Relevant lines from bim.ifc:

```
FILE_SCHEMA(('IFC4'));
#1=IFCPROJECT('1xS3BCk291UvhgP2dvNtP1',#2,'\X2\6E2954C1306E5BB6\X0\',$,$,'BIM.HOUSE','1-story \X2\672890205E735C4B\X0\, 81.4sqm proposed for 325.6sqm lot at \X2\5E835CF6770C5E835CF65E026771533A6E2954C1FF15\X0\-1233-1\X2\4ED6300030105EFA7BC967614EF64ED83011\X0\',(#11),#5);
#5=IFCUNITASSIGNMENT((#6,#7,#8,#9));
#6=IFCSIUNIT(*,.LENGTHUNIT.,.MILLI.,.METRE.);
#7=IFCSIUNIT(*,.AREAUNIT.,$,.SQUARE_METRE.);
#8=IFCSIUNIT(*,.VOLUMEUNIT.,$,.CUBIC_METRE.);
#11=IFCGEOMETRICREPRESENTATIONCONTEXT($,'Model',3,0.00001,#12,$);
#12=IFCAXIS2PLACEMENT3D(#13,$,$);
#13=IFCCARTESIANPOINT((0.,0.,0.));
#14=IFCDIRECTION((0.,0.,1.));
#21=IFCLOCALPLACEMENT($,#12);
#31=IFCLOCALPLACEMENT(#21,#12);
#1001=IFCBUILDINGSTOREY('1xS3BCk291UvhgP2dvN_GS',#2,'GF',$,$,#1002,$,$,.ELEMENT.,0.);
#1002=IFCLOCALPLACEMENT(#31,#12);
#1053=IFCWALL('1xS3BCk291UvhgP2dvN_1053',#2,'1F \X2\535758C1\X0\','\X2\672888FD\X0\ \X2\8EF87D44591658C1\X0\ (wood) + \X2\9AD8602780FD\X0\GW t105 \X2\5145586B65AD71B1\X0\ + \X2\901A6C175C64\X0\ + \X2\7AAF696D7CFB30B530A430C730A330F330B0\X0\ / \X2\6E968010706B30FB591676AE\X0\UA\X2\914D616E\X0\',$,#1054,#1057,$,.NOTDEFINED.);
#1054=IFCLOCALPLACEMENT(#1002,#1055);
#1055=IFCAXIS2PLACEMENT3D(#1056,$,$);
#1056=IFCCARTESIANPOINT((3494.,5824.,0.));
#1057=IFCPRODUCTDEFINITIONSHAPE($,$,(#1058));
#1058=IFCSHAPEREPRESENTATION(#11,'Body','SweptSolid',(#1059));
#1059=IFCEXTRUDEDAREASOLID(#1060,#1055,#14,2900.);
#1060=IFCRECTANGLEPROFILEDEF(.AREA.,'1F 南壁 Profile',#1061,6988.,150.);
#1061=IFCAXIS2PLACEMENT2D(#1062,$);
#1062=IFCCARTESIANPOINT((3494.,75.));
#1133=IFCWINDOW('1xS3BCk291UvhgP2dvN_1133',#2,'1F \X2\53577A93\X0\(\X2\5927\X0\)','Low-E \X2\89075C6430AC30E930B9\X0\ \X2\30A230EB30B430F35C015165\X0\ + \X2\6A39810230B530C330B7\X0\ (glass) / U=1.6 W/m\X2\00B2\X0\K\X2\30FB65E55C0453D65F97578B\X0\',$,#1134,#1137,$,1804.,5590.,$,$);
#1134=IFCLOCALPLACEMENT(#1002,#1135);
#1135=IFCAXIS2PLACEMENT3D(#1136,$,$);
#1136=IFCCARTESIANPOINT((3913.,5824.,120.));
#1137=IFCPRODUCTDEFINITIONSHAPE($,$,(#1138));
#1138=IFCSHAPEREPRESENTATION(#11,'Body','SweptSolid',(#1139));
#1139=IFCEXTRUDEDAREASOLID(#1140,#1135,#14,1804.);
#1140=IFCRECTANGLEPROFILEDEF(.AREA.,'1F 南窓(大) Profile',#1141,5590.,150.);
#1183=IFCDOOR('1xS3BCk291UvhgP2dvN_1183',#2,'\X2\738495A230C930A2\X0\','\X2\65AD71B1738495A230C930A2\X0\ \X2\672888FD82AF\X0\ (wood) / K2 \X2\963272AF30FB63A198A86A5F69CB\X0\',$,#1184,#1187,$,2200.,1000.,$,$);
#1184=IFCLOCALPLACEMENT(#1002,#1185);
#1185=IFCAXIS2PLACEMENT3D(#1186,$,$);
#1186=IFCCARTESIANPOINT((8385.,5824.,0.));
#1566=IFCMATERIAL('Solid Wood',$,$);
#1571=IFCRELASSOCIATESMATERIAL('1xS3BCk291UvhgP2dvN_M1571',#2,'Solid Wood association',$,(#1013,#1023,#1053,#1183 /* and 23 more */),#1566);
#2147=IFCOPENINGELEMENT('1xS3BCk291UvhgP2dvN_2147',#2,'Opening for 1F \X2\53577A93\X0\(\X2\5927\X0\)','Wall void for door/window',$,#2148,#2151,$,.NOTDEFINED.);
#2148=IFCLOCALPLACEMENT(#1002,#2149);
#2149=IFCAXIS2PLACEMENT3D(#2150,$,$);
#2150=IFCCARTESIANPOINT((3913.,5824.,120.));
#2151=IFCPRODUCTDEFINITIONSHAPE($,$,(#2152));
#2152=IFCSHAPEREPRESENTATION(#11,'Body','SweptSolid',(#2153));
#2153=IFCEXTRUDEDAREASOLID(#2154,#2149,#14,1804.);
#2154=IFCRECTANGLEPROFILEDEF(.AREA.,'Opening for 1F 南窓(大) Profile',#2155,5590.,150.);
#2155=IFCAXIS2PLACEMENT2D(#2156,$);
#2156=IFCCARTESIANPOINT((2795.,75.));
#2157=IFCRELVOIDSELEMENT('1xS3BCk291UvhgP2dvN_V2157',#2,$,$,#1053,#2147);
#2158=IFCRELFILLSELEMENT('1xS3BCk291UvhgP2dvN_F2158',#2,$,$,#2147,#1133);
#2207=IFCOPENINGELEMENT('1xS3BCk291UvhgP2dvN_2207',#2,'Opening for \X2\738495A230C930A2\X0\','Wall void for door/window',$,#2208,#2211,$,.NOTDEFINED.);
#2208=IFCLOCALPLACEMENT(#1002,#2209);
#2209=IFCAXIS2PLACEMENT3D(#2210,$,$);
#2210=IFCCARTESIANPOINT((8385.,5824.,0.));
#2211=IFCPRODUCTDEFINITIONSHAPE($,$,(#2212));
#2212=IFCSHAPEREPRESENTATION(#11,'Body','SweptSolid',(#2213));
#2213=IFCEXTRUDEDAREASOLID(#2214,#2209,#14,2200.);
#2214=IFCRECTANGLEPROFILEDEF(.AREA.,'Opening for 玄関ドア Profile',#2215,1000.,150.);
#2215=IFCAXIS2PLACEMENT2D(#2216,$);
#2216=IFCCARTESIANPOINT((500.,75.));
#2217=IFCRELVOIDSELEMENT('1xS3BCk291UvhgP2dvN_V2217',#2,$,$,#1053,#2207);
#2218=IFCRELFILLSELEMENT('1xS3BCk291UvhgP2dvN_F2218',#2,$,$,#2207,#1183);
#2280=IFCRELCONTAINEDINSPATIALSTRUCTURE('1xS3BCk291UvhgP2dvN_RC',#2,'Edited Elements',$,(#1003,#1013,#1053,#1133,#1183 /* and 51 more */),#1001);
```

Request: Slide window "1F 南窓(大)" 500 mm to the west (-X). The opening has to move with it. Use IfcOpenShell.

```python
import ifcopenshell
import ifcopenshell.api.geometry
import ifcopenshell.util.placement

model = ifcopenshell.open("bim.ifc")

window = model.by_id(1133)
opening = window.FillsVoids[0].RelatingOpeningElement
wall = opening.VoidsElements[0].RelatingBuildingElement

wall_matrix = ifcopenshell.util.placement.get_local_placement(wall.ObjectPlacement)
shift = wall_matrix[:3, 0] * -500.0
before = ifcopenshell.util.placement.get_local_placement(window.ObjectPlacement)[:3, 3].copy()

# The window is not placed relative to its opening, so move both.
for product in (opening, window):
    matrix = ifcopenshell.util.placement.get_local_placement(product.ObjectPlacement)
    matrix[:3, 3] += shift
    ifcopenshell.api.geometry.edit_object_placement(model, product=product, matrix=matrix, is_si=False)

after = ifcopenshell.util.placement.get_local_placement(window.ObjectPlacement)[:3, 3]
print("window moved by", (after - before).round(3) + 0.0)

model.write("bim_v2.ifc")
```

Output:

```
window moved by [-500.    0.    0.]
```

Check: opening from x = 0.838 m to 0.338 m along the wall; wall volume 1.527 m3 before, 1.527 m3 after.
